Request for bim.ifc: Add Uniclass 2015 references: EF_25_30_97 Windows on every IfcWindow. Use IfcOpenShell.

First a look at what the model holds.

```python
import ifcopenshell

model = ifcopenshell.open("bim.ifc")
print(model.schema)
print("classifications:", [c.Name for c in model.by_type("IfcClassification")])
for ifc_class in ("IfcDoor", "IfcRoof", "IfcStair", "IfcWall", "IfcWindow"):
    print(ifc_class, len(model.by_type(ifc_class)))
```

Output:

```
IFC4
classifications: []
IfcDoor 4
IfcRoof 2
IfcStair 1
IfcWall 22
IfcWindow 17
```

```python
import ifcopenshell
import ifcopenshell.api.classification

model = ifcopenshell.open("bim.ifc")

system = ifcopenshell.api.classification.add_classification(model, classification="Uniclass 2015")

codes = {
    "IfcWindow": ("EF_25_30_97", "Windows"),
}
for ifc_class, (code, name) in codes.items():
    products = model.by_type(ifc_class)
    ifcopenshell.api.classification.add_reference(
        model, products=products, classification=system, identification=code, name=name
    )
    print(code, len(products))

model.write("bim_updated.ifc")
```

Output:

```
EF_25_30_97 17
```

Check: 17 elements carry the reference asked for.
